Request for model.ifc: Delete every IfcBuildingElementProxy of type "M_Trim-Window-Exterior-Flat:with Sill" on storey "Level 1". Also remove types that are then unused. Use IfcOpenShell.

First a look at what the model holds.

```python
import ifcopenshell
import ifcopenshell.util.element

model = ifcopenshell.open("model.ifc")
print(model.schema)
storey = next(s for s in model.by_type("IfcBuildingStorey") if s.Name == "Level 1")
proxies = [e for e in ifcopenshell.util.element.get_decomposition(storey) if e.is_a("IfcBuildingElementProxy")]
seen = {}
for e in proxies:
    element_type = ifcopenshell.util.element.get_type(e)
    name = element_type.Name if element_type not in (None, e) else None
    seen[name] = seen.get(name, 0) + 1
for name, count in sorted(seen.items(), key=str):
    print(count, "x", name)
```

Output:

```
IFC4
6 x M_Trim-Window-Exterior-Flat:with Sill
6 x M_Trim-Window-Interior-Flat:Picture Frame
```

```python
import ifcopenshell
import ifcopenshell.api.root
import ifcopenshell.util.element

model = ifcopenshell.open("model.ifc")

storey = next(s for s in model.by_type("IfcBuildingStorey") if s.Name == "Level 1")
proxies = [e for e in ifcopenshell.util.element.get_decomposition(storey) if e.is_a("IfcBuildingElementProxy")]
targets = [e for e in proxies if (t := ifcopenshell.util.element.get_type(e)) not in (None, e) and t.Name == "M_Trim-Window-Exterior-Flat:with Sill"]
types = {ifcopenshell.util.element.get_type(e) for e in targets} - {None, *targets}

for e in targets:
    ifcopenshell.api.root.remove_product(model, product=e)
print(len(targets), "removed")

unused = [t for t in types if not ifcopenshell.util.element.get_types(t)]
for t in unused:
    ifcopenshell.api.root.remove_product(model, product=t)
print(len(unused), "unused types removed")

model.write("model_v2.ifc")
```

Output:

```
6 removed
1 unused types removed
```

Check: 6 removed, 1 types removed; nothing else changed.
